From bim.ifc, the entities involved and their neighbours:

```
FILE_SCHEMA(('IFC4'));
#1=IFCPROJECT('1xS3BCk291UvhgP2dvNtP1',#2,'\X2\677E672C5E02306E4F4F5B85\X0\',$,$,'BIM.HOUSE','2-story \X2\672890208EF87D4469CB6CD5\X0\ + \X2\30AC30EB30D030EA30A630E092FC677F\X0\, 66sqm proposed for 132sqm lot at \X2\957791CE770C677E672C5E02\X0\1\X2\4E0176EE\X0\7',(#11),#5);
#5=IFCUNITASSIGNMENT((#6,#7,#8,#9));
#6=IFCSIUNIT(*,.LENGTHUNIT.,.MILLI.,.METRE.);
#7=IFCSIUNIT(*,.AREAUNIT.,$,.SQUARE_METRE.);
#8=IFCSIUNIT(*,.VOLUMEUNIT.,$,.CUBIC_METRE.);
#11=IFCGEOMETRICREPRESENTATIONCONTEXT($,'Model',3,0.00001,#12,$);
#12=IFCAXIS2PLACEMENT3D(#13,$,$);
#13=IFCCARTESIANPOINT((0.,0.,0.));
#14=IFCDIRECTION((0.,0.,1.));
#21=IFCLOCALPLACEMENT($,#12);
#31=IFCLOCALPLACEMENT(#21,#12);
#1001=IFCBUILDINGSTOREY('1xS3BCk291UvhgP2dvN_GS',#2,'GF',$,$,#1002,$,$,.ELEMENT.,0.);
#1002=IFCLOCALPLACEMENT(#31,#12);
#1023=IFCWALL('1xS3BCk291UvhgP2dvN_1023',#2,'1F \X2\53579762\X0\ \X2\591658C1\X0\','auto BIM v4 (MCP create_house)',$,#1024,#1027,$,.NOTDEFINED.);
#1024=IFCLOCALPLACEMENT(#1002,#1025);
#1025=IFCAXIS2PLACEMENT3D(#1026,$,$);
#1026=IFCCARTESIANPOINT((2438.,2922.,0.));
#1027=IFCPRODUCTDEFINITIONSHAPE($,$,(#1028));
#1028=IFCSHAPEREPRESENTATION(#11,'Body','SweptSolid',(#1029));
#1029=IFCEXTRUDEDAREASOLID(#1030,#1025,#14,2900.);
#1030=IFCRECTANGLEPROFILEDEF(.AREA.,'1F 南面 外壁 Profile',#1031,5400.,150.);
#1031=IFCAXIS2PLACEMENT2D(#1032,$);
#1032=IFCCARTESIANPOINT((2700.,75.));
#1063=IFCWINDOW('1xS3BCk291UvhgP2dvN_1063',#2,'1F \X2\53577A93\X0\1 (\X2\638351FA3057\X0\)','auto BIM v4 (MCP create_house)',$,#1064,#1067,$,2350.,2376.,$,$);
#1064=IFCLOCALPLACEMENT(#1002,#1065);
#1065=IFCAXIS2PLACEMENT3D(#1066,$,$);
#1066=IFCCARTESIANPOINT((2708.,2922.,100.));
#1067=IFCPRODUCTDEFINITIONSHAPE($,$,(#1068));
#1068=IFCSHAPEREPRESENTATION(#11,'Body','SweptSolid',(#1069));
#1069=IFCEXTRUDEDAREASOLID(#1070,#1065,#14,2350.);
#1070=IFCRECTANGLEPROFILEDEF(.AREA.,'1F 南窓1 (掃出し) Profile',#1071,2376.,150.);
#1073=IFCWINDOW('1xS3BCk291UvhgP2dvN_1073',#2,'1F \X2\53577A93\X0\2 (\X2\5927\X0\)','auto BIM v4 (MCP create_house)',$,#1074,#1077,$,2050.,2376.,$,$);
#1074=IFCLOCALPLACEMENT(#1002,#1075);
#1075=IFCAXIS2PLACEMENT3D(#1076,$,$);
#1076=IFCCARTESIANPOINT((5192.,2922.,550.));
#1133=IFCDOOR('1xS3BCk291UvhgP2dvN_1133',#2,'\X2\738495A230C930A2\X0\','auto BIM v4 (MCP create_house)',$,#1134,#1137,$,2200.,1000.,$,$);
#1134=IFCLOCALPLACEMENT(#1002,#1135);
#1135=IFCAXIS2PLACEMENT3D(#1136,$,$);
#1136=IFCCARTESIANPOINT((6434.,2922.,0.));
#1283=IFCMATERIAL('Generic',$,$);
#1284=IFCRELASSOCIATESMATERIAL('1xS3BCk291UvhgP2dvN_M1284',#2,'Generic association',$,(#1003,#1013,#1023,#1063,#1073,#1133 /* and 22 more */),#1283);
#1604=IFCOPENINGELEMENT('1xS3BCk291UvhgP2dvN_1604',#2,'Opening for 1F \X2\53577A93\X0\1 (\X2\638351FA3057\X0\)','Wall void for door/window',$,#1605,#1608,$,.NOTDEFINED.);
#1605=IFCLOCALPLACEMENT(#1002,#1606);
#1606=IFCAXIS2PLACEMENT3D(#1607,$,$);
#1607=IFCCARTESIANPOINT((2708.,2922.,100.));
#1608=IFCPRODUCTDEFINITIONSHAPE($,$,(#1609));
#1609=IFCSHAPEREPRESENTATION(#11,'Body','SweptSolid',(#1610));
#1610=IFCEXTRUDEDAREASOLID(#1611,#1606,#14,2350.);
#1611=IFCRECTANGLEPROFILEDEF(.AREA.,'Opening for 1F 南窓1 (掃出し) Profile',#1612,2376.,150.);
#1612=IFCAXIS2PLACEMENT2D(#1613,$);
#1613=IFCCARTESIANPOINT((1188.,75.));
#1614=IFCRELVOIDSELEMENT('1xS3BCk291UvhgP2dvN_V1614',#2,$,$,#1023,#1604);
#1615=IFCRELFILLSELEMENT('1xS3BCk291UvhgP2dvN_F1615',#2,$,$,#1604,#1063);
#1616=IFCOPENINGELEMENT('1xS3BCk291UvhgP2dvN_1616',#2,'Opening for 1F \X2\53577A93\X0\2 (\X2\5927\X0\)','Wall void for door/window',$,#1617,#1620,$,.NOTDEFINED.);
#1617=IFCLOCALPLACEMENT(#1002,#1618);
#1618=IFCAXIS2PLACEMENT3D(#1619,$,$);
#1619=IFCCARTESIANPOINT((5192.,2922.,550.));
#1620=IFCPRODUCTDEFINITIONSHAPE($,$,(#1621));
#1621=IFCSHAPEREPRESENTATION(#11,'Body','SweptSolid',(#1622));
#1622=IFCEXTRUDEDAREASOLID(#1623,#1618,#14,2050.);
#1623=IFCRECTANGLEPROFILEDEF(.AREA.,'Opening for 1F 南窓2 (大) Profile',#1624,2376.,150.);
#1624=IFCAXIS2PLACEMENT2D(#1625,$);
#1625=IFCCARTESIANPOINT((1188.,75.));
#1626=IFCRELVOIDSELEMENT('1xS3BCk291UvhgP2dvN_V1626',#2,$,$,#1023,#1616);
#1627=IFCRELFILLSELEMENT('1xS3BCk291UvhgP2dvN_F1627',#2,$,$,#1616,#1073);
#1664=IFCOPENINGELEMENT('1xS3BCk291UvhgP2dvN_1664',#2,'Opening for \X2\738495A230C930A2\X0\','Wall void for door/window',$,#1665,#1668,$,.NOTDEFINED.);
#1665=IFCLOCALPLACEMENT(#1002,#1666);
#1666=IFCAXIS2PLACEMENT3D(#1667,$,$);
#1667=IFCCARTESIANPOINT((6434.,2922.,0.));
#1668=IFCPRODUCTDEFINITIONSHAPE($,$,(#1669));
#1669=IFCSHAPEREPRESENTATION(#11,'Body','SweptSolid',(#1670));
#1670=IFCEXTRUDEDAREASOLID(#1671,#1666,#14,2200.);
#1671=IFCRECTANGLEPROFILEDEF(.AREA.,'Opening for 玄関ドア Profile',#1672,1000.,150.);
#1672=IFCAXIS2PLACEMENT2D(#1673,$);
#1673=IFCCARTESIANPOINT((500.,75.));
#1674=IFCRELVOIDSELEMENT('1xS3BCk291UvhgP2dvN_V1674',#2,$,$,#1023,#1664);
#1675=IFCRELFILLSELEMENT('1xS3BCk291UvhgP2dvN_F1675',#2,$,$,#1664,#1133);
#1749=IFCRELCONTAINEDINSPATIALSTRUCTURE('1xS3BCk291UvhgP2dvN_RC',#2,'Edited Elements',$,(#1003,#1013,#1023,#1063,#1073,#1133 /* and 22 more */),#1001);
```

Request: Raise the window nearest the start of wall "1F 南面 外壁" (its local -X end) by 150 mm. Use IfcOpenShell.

```python
import numpy as np
import ifcopenshell
import ifcopenshell.api.geometry
import ifcopenshell.util.placement
import ifcopenshell.util.unit

model = ifcopenshell.open("bim.ifc")
unit_scale = ifcopenshell.util.unit.calculate_unit_scale(model)

window = model.by_guid("1xS3BCk291UvhgP2dvN_1063")
opening = window.FillsVoids[0].RelatingOpeningElement
dz = 150.0

shift = np.array([0.0, 0.0, dz])
# The window is not placed relative to its opening, so move both.
for product in (opening, window):
    matrix = ifcopenshell.util.placement.get_local_placement(product.ObjectPlacement)
    matrix[:3, 3] += shift
    ifcopenshell.api.geometry.edit_object_placement(model, product=product, matrix=matrix, is_si=False)

print(f"moved by {dz * unit_scale:+.3f} m")

model.write("bim_updated.ifc")
```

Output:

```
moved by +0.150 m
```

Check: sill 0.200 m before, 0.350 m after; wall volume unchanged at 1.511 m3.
